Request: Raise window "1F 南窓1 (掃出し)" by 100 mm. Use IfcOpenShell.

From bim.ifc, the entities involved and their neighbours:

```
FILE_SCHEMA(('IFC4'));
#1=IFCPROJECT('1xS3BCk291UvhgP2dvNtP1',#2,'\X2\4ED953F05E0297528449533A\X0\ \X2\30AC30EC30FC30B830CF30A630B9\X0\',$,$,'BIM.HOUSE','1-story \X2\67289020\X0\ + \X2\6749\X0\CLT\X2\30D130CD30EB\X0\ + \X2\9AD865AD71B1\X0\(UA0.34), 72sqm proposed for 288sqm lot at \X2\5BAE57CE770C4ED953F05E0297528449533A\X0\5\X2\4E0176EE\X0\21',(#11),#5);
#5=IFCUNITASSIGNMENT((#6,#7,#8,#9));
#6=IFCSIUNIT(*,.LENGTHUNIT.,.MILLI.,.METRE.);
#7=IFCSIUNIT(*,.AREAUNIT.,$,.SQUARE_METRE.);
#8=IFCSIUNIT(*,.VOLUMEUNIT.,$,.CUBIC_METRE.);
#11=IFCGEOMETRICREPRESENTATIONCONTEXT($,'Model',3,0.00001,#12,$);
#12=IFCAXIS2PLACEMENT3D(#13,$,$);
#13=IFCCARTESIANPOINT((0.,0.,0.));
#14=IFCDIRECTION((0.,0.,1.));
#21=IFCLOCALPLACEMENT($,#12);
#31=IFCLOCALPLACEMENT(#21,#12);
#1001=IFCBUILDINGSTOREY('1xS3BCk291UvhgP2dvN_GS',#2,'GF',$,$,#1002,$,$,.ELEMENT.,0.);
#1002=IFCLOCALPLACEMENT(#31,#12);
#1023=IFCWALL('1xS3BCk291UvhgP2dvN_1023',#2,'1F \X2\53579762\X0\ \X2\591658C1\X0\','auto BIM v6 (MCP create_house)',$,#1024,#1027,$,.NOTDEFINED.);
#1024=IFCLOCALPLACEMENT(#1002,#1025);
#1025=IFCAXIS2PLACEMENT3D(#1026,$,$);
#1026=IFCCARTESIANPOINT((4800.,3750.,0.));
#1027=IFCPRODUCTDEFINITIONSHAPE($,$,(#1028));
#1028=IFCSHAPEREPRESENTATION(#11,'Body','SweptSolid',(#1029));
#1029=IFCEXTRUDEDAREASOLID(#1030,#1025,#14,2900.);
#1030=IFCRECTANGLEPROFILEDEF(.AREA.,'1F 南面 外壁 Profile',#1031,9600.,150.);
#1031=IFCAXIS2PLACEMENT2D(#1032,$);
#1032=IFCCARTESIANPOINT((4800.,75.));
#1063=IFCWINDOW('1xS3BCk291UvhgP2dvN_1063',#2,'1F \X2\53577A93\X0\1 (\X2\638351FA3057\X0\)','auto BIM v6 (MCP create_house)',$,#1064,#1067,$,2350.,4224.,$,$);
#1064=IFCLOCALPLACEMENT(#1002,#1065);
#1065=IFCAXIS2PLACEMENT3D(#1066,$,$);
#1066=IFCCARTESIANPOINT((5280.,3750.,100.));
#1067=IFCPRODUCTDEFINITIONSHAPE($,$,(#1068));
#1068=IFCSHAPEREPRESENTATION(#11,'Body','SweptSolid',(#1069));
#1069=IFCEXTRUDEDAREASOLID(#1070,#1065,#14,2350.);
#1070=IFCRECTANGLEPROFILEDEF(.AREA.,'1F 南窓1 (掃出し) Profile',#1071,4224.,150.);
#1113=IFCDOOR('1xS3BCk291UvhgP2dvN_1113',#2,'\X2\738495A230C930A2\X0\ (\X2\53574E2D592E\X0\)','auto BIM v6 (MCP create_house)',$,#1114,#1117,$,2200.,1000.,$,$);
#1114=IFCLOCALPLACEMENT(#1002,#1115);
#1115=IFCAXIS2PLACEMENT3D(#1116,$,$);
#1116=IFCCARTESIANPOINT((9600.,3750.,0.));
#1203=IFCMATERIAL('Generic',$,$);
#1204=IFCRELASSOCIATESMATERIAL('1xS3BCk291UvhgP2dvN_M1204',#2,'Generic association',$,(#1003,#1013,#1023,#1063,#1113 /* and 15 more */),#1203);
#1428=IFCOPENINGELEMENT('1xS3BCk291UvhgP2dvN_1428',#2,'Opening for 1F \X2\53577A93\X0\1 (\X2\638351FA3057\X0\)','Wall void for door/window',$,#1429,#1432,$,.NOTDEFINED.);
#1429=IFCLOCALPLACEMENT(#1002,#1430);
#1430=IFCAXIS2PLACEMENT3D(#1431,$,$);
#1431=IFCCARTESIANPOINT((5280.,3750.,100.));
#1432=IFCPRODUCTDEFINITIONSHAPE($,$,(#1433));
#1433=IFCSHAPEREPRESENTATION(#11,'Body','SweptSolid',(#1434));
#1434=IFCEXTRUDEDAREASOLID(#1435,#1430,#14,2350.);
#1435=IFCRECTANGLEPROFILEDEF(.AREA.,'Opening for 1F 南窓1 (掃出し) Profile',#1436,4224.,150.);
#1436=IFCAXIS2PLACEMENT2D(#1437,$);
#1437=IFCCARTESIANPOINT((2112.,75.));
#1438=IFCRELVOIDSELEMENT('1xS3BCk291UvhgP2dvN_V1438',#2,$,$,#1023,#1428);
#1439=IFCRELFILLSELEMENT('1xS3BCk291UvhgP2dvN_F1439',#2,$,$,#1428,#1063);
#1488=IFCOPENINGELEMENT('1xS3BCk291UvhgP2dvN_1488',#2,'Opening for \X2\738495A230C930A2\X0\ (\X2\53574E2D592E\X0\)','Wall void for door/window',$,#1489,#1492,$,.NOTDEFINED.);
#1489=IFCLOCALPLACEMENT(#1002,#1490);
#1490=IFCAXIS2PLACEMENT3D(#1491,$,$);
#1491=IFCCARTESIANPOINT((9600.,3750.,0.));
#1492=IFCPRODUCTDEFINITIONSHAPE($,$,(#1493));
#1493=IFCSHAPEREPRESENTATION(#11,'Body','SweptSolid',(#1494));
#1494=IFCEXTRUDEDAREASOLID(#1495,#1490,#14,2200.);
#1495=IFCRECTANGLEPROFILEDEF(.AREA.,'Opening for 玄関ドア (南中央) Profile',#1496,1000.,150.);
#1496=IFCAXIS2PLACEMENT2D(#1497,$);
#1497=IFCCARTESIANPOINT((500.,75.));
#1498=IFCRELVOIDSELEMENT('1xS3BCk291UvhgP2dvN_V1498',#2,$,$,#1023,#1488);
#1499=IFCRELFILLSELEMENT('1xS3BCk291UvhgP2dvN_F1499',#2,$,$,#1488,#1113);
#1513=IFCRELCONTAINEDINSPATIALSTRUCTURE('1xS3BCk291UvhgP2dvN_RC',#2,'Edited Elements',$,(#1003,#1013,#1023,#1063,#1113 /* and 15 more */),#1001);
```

```python
import numpy as np
import ifcopenshell
import ifcopenshell.api.geometry
import ifcopenshell.util.placement
import ifcopenshell.util.unit

model = ifcopenshell.open("bim.ifc")
unit_scale = ifcopenshell.util.unit.calculate_unit_scale(model)

window = model.by_id(1063)
opening = window.FillsVoids[0].RelatingOpeningElement
dz = 0.1 / unit_scale

shift = np.array([0.0, 0.0, dz])
# The window is not placed relative to its opening, so move both.
for product in (opening, window):
    matrix = ifcopenshell.util.placement.get_local_placement(product.ObjectPlacement)
    matrix[:3, 3] += shift
    ifcopenshell.api.geometry.edit_object_placement(model, product=product, matrix=matrix, is_si=False)

print(f"moved by {dz * unit_scale:+.3f} m")

model.write("bim_updated.ifc")
```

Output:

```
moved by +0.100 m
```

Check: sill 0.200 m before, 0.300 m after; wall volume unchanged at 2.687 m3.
